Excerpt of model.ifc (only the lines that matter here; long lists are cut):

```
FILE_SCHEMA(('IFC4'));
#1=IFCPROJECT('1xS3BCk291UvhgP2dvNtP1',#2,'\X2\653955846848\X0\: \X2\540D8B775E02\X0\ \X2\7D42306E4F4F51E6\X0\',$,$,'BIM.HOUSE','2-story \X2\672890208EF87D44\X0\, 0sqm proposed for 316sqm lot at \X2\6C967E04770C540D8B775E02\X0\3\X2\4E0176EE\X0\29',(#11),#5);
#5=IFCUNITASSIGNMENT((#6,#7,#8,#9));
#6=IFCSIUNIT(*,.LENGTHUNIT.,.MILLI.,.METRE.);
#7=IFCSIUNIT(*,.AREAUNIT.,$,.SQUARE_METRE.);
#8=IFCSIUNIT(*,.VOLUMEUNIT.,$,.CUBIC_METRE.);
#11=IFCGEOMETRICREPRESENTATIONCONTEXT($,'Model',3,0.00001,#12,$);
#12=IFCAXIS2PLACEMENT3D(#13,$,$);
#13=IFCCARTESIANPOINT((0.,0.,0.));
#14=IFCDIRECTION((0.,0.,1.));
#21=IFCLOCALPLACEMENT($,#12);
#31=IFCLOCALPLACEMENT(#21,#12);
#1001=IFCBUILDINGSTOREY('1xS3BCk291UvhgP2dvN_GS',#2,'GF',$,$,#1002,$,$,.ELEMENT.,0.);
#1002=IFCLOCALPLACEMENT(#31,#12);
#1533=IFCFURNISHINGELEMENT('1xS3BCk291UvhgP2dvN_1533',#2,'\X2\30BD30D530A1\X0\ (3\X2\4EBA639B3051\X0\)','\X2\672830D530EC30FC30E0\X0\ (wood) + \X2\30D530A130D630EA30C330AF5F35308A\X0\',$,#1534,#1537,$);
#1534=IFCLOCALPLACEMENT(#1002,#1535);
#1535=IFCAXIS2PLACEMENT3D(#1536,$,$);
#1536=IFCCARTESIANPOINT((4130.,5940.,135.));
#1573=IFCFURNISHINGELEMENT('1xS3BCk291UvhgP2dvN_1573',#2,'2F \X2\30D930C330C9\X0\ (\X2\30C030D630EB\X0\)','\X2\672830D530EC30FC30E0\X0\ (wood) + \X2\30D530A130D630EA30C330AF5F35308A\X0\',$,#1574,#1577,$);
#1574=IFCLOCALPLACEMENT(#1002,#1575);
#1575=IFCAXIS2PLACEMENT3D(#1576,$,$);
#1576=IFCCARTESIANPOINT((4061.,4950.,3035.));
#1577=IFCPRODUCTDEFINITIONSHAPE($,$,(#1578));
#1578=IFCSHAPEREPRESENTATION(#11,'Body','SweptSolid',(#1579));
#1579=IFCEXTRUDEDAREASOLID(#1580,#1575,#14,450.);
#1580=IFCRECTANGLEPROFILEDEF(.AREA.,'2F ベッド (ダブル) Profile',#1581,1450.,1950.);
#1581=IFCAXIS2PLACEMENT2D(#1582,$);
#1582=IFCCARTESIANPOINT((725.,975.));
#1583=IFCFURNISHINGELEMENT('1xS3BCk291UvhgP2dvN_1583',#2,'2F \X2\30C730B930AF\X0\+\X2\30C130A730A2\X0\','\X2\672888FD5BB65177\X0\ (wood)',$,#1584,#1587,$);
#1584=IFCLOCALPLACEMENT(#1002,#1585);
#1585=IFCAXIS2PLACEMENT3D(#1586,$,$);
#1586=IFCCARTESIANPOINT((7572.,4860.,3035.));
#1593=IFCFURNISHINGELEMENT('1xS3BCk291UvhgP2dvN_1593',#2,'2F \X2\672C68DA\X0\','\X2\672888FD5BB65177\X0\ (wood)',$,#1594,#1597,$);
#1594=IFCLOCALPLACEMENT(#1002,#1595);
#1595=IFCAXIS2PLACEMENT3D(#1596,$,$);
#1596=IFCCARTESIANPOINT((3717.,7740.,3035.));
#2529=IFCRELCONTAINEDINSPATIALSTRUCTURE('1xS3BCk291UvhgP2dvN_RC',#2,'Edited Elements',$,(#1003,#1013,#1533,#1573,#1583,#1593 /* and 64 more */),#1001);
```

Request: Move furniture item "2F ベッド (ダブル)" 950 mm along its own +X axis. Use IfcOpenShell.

```python
import ifcopenshell
import ifcopenshell.api.geometry
import ifcopenshell.util.placement
import ifcopenshell.util.unit

model = ifcopenshell.open("model.ifc")
unit_scale = ifcopenshell.util.unit.calculate_unit_scale(model)

item = model.by_guid("1xS3BCk291UvhgP2dvN_1573")
matrix = ifcopenshell.util.placement.get_local_placement(item.ObjectPlacement)
matrix[:3, 3] += matrix[:3, 0] * 0.95 / unit_scale
ifcopenshell.api.geometry.edit_object_placement(model, product=item, matrix=matrix, is_si=False)

print(ifcopenshell.util.placement.get_local_placement(item.ObjectPlacement).round(3) + 0.0)

model.write("model_rev.ifc")
```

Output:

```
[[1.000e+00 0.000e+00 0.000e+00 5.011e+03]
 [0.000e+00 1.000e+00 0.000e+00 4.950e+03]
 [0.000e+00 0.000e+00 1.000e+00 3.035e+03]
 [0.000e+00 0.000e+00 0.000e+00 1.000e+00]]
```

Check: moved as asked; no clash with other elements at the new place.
